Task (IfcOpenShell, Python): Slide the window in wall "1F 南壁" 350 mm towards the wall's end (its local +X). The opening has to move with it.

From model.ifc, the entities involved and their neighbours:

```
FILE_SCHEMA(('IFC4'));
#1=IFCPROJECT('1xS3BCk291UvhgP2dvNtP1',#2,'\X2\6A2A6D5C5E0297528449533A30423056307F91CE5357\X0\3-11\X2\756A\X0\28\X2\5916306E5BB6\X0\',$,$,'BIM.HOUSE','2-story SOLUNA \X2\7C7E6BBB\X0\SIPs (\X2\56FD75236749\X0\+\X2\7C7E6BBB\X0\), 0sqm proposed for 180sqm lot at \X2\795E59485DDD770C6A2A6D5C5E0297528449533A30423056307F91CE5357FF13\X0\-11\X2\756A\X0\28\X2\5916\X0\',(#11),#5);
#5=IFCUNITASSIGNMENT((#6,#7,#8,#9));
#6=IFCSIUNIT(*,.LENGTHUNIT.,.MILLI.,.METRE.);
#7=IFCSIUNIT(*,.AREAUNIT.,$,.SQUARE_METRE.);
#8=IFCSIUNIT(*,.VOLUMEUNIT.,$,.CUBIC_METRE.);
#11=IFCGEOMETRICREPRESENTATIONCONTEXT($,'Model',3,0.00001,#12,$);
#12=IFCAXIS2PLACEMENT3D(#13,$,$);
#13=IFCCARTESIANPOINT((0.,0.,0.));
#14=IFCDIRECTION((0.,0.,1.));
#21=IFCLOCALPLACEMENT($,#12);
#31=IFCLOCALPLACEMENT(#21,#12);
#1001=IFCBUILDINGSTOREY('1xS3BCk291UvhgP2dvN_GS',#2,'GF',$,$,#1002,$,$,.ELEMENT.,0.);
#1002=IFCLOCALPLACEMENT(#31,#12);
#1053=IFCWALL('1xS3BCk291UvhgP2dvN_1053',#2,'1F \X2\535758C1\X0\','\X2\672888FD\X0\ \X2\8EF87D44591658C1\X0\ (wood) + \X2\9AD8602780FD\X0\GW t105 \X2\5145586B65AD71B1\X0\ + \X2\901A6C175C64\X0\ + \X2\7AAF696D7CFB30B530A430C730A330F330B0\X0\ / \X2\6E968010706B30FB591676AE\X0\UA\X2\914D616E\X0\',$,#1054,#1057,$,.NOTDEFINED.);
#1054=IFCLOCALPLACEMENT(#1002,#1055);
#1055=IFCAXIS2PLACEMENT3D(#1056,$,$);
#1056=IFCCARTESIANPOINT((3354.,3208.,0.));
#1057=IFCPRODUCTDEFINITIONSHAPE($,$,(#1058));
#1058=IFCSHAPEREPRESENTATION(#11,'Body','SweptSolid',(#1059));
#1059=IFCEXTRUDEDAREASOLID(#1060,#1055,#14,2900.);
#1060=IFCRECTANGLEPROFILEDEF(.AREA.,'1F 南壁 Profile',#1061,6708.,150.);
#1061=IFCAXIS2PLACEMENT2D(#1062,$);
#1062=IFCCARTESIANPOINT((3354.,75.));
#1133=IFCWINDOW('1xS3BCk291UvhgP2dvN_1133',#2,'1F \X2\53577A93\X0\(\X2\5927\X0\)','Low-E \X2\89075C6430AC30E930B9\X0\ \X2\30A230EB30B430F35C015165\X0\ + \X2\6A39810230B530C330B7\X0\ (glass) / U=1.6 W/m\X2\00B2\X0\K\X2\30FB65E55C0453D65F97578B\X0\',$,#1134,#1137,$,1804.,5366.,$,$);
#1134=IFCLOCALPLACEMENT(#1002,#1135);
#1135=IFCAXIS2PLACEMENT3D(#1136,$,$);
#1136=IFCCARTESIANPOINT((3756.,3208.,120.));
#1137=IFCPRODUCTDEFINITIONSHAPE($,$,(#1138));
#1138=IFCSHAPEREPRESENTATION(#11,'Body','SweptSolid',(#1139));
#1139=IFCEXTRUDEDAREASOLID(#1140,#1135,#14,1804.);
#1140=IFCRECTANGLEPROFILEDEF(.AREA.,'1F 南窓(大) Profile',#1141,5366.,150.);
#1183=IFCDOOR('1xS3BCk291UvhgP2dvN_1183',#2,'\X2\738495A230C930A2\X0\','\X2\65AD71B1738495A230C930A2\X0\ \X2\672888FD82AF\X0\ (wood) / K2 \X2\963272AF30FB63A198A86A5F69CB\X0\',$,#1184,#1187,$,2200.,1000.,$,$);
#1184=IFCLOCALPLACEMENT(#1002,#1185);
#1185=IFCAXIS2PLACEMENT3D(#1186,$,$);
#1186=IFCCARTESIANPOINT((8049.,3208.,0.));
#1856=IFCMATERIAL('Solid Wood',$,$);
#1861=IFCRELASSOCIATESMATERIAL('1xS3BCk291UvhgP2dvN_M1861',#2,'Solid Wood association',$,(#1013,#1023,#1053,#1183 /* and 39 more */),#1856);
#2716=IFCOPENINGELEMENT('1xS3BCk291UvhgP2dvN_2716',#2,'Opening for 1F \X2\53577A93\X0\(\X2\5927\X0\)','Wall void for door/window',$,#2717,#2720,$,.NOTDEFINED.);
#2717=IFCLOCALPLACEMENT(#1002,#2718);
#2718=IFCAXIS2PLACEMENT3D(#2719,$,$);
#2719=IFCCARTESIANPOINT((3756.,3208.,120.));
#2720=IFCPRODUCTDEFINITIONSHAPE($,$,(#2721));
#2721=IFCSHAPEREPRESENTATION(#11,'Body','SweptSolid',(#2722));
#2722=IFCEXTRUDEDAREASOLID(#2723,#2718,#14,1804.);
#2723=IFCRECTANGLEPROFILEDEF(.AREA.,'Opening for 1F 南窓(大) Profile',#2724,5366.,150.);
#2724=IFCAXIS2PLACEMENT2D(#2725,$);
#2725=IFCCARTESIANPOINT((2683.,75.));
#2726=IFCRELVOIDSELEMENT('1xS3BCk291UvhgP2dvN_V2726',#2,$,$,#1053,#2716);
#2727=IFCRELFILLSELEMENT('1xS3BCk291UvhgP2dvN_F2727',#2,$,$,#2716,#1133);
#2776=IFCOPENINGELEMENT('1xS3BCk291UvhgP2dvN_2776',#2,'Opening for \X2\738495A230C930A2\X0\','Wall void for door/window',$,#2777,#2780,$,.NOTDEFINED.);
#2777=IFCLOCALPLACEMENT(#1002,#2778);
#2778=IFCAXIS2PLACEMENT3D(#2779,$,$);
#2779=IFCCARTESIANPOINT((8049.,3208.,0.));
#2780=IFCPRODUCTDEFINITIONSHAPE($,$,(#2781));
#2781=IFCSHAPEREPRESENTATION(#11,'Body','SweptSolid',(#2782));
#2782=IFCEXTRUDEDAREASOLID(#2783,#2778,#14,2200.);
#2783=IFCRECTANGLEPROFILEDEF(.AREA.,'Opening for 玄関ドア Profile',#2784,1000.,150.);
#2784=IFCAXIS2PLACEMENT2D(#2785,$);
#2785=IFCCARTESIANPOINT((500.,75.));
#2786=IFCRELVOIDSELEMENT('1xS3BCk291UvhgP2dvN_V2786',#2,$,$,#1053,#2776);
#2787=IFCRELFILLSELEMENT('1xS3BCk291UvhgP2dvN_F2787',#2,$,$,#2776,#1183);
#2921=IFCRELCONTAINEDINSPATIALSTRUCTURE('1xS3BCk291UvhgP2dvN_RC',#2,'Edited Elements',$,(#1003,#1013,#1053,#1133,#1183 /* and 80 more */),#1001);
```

```python
import ifcopenshell
import ifcopenshell.api.geometry
import ifcopenshell.util.placement
import ifcopenshell.util.unit

model = ifcopenshell.open("model.ifc")
unit_scale = ifcopenshell.util.unit.calculate_unit_scale(model)

window = model.by_id(1133)
opening = window.FillsVoids[0].RelatingOpeningElement
wall = opening.VoidsElements[0].RelatingBuildingElement

wall_matrix = ifcopenshell.util.placement.get_local_placement(wall.ObjectPlacement)
shift = wall_matrix[:3, 0] * 0.35 / unit_scale
before = ifcopenshell.util.placement.get_local_placement(window.ObjectPlacement)[:3, 3].copy()

# The window is not placed relative to its opening, so move both.
for product in (opening, window):
    matrix = ifcopenshell.util.placement.get_local_placement(product.ObjectPlacement)
    matrix[:3, 3] += shift
    ifcopenshell.api.geometry.edit_object_placement(model, product=product, matrix=matrix, is_si=False)

after = ifcopenshell.util.placement.get_local_placement(window.ObjectPlacement)[:3, 3]
print("window moved by", (after - before).round(3) + 0.0)

model.write("model_v2.ifc")
```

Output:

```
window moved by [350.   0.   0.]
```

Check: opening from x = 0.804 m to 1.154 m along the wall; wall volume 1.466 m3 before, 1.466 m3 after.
